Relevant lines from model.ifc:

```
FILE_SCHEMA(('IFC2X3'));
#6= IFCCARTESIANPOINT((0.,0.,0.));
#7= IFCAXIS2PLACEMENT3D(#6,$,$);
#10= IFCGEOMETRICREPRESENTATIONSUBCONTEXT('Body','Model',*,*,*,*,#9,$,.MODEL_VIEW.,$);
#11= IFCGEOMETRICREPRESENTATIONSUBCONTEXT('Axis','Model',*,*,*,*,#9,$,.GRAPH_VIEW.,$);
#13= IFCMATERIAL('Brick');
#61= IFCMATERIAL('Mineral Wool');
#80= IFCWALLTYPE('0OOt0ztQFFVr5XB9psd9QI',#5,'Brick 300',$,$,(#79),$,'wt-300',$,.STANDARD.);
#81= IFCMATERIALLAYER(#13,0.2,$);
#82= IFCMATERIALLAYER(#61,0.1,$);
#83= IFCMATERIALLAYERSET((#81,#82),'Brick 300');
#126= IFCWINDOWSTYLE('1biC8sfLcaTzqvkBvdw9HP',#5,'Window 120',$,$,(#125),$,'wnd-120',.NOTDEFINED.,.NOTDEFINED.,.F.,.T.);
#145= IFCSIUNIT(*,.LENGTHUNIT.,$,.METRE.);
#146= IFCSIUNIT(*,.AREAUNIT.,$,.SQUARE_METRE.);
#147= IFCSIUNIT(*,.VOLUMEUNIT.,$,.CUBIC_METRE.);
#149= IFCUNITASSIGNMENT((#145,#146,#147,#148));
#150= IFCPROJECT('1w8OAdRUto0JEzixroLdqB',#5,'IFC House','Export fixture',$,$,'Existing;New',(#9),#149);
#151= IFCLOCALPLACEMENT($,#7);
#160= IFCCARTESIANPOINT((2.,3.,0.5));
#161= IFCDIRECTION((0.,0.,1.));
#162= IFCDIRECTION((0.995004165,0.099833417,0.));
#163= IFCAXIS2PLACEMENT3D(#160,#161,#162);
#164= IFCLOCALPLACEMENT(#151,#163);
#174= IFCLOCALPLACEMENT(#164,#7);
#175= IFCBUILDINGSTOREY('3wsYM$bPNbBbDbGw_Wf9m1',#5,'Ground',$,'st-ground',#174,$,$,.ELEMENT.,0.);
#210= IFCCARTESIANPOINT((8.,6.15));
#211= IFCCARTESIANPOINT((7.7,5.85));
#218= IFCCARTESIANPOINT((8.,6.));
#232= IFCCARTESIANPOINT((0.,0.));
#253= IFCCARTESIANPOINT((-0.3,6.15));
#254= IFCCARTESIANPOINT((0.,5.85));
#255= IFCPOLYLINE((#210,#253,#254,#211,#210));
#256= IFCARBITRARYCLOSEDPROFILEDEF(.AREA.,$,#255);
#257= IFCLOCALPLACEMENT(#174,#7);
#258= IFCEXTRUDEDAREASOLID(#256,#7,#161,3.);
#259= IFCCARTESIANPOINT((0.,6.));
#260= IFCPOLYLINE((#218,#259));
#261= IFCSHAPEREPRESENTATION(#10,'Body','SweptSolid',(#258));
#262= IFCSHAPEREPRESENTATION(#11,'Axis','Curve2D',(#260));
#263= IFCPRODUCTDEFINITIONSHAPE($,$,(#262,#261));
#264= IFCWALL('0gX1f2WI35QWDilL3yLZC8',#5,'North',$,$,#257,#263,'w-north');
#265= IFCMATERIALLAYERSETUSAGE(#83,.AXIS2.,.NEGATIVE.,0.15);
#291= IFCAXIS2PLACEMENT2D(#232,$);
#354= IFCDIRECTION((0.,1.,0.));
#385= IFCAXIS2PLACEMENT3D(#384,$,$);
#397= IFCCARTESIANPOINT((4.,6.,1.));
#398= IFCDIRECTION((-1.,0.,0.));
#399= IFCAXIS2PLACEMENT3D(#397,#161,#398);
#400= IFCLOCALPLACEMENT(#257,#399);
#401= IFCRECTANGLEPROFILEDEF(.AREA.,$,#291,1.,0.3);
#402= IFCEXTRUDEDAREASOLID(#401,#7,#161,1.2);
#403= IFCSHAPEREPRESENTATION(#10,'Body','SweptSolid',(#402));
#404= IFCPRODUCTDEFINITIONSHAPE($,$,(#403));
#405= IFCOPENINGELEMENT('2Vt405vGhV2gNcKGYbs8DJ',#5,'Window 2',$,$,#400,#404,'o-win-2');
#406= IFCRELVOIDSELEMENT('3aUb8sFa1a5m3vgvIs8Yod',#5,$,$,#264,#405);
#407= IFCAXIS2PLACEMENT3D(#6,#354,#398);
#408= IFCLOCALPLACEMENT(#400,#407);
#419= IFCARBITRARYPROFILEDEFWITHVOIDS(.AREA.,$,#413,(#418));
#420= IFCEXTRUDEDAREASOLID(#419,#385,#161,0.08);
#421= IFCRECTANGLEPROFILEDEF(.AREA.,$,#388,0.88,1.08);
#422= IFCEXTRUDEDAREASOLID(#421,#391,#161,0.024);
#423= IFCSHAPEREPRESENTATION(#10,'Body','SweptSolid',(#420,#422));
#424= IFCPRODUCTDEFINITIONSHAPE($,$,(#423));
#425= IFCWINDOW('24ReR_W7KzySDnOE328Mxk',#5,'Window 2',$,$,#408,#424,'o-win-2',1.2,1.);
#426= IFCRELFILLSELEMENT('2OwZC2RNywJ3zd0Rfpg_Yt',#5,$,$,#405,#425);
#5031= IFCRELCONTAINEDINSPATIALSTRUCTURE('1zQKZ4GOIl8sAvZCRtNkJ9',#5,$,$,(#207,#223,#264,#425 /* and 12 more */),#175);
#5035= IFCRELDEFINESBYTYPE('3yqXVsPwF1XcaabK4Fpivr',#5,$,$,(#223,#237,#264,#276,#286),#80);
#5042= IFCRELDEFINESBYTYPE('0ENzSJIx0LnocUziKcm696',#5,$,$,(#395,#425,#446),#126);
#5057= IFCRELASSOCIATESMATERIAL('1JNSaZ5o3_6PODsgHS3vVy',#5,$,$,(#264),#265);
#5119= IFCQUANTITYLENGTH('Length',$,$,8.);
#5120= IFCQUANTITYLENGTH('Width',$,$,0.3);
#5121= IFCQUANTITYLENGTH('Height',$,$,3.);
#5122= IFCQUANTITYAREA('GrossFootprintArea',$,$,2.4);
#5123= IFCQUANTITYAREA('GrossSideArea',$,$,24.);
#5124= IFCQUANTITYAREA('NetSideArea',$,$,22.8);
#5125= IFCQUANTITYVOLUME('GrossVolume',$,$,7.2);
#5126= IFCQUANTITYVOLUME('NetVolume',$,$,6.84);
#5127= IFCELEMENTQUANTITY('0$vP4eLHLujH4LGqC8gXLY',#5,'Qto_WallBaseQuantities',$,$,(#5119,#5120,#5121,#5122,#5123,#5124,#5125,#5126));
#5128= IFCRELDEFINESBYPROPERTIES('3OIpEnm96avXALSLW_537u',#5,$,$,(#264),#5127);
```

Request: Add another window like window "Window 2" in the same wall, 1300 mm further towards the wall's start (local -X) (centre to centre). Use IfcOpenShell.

```python
import ifcopenshell
import ifcopenshell.api.feature
import ifcopenshell.api.geometry
import ifcopenshell.api.pset
import ifcopenshell.api.root
import ifcopenshell.geom
import ifcopenshell.util.element
import ifcopenshell.util.placement
import ifcopenshell.util.shape
import ifcopenshell.util.unit

model = ifcopenshell.open("model.ifc")
unit_scale = ifcopenshell.util.unit.calculate_unit_scale(model)
area_scale = ifcopenshell.util.unit.calculate_unit_scale(model, "AREAUNIT")
volume_scale = ifcopenshell.util.unit.calculate_unit_scale(model, "VOLUMEUNIT")
settings = ifcopenshell.geom.settings()


def volume(element):
    """Net volume in cubic metres, openings subtracted."""
    shape = ifcopenshell.geom.create_shape(settings, element)
    return ifcopenshell.util.shape.get_volume(shape.geometry)


def reuse_history(source, copy):
    """copy_class also copies each property set's owner history, people and application; keep the originals."""
    for rel in copy.IsDefinedBy:
        if rel.is_a("IfcRelDefinesByProperties") and (history := rel.RelatingPropertyDefinition.OwnerHistory):
            rel.RelatingPropertyDefinition.OwnerHistory = source.OwnerHistory
            ifcopenshell.util.element.remove_deep2(model, history)


window = model.by_guid("24ReR_W7KzySDnOE328Mxk")
opening = window.FillsVoids[0].RelatingOpeningElement
wall = opening.VoidsElements[0].RelatingBuildingElement
before = volume(wall)
shift = ifcopenshell.util.placement.get_local_placement(wall.ObjectPlacement)[:3, 0] * -1.3 / unit_scale

# copy_class copies the void relationship, type, container and properties, but no geometry.
new_opening = ifcopenshell.api.root.copy_class(model, product=opening)
new_opening.Representation = ifcopenshell.util.element.copy_deep(
    model, opening.Representation, exclude=["IfcGeometricRepresentationContext", "IfcRepresentationMap"]
)
new_opening.Tag = None
new_window = ifcopenshell.api.root.copy_class(model, product=window)
new_window.Representation = ifcopenshell.util.element.copy_deep(
    model, window.Representation, exclude=["IfcGeometricRepresentationContext", "IfcRepresentationMap"]
)
new_window.Tag = None
reuse_history(window, new_window)
fills = ifcopenshell.api.feature.add_filling(model, opening=new_opening, element=new_window)
fills.OwnerHistory = new_window.OwnerHistory  # required in IFC2X3

for old, new in ((opening, new_opening), (window, new_window)):
    matrix = ifcopenshell.util.placement.get_local_placement(old.ObjectPlacement)
    matrix[:3, 3] += shift
    ifcopenshell.api.geometry.edit_object_placement(model, product=new, matrix=matrix, is_si=False)

after = volume(wall)
thickness = 0.3  # wall thickness in metres

# Update the wall's stored quantities.
qto = model.by_id(ifcopenshell.util.element.get_pset(wall, "Qto_WallBaseQuantities", should_inherit=False)["id"])
ifcopenshell.api.pset.edit_qto(model, qto=qto, properties={
    "NetSideArea": after / thickness / area_scale,
    "NetVolume": after / volume_scale,
})

print(f"wall volume {before:.3f} -> {after:.3f} m3")

model.write("model_v2.ifc")
```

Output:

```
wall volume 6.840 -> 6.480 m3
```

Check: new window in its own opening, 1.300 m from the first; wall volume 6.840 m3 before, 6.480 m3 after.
